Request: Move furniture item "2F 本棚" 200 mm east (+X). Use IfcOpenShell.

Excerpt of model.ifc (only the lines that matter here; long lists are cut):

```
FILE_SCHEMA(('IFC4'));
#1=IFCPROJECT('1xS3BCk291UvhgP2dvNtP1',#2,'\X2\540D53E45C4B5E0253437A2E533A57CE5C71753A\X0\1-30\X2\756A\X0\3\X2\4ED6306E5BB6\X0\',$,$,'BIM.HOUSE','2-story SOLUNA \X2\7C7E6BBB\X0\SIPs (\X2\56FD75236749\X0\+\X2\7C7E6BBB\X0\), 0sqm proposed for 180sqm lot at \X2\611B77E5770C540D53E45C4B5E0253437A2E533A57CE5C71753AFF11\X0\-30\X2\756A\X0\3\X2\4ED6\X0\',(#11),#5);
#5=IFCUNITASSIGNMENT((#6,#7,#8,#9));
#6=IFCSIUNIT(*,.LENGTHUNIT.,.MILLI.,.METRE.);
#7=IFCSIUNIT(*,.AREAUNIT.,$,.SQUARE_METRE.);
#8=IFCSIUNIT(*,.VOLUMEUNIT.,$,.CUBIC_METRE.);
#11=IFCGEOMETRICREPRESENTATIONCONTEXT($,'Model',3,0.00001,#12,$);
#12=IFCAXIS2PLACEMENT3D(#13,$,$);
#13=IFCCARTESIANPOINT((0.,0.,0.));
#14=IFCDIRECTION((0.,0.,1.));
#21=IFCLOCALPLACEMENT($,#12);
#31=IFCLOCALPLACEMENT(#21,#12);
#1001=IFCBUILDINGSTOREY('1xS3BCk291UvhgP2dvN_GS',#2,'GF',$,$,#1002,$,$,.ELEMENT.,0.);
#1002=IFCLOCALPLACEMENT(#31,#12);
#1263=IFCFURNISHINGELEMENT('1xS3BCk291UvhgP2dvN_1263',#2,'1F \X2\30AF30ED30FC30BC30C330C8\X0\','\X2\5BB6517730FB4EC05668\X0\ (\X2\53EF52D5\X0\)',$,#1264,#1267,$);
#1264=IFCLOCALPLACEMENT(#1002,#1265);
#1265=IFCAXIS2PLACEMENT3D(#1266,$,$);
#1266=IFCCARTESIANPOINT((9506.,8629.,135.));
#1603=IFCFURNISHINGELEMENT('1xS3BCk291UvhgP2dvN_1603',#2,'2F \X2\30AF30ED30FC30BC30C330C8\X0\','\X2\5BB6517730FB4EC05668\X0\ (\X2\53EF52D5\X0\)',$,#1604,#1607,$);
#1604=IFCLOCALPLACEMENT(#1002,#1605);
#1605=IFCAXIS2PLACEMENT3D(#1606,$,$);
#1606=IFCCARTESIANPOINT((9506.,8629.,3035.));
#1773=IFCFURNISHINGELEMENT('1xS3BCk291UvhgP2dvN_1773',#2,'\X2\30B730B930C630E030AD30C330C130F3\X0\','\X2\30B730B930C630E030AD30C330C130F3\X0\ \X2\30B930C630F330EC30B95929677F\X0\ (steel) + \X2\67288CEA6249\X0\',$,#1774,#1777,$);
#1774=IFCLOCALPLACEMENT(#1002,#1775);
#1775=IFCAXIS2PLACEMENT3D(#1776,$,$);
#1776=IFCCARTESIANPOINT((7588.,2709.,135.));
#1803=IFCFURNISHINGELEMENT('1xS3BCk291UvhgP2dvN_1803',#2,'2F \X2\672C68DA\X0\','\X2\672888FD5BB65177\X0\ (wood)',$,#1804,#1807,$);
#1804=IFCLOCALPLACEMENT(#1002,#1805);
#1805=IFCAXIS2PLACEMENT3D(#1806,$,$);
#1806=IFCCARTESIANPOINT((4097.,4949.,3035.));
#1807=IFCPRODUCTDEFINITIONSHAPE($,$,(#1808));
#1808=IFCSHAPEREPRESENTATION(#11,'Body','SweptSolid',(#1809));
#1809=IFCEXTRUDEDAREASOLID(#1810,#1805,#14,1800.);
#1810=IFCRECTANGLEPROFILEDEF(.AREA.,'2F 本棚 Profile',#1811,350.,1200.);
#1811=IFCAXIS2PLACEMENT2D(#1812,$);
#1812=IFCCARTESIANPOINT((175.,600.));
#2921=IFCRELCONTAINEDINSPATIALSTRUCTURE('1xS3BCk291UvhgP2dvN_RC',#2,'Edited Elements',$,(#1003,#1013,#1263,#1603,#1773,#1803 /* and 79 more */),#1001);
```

```python
import ifcopenshell
import ifcopenshell.api.geometry
import ifcopenshell.util.placement

model = ifcopenshell.open("model.ifc")

item = model.by_guid("1xS3BCk291UvhgP2dvN_1803")
matrix = ifcopenshell.util.placement.get_local_placement(item.ObjectPlacement)
matrix[0, 3] += 200.0
ifcopenshell.api.geometry.edit_object_placement(model, product=item, matrix=matrix, is_si=False)

print(ifcopenshell.util.placement.get_local_placement(item.ObjectPlacement).round(3) + 0.0)

model.write("model_edited.ifc")
```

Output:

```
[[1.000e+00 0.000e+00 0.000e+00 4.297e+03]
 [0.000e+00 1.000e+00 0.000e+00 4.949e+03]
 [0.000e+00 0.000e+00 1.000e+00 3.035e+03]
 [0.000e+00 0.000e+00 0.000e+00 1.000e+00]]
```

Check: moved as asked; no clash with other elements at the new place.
